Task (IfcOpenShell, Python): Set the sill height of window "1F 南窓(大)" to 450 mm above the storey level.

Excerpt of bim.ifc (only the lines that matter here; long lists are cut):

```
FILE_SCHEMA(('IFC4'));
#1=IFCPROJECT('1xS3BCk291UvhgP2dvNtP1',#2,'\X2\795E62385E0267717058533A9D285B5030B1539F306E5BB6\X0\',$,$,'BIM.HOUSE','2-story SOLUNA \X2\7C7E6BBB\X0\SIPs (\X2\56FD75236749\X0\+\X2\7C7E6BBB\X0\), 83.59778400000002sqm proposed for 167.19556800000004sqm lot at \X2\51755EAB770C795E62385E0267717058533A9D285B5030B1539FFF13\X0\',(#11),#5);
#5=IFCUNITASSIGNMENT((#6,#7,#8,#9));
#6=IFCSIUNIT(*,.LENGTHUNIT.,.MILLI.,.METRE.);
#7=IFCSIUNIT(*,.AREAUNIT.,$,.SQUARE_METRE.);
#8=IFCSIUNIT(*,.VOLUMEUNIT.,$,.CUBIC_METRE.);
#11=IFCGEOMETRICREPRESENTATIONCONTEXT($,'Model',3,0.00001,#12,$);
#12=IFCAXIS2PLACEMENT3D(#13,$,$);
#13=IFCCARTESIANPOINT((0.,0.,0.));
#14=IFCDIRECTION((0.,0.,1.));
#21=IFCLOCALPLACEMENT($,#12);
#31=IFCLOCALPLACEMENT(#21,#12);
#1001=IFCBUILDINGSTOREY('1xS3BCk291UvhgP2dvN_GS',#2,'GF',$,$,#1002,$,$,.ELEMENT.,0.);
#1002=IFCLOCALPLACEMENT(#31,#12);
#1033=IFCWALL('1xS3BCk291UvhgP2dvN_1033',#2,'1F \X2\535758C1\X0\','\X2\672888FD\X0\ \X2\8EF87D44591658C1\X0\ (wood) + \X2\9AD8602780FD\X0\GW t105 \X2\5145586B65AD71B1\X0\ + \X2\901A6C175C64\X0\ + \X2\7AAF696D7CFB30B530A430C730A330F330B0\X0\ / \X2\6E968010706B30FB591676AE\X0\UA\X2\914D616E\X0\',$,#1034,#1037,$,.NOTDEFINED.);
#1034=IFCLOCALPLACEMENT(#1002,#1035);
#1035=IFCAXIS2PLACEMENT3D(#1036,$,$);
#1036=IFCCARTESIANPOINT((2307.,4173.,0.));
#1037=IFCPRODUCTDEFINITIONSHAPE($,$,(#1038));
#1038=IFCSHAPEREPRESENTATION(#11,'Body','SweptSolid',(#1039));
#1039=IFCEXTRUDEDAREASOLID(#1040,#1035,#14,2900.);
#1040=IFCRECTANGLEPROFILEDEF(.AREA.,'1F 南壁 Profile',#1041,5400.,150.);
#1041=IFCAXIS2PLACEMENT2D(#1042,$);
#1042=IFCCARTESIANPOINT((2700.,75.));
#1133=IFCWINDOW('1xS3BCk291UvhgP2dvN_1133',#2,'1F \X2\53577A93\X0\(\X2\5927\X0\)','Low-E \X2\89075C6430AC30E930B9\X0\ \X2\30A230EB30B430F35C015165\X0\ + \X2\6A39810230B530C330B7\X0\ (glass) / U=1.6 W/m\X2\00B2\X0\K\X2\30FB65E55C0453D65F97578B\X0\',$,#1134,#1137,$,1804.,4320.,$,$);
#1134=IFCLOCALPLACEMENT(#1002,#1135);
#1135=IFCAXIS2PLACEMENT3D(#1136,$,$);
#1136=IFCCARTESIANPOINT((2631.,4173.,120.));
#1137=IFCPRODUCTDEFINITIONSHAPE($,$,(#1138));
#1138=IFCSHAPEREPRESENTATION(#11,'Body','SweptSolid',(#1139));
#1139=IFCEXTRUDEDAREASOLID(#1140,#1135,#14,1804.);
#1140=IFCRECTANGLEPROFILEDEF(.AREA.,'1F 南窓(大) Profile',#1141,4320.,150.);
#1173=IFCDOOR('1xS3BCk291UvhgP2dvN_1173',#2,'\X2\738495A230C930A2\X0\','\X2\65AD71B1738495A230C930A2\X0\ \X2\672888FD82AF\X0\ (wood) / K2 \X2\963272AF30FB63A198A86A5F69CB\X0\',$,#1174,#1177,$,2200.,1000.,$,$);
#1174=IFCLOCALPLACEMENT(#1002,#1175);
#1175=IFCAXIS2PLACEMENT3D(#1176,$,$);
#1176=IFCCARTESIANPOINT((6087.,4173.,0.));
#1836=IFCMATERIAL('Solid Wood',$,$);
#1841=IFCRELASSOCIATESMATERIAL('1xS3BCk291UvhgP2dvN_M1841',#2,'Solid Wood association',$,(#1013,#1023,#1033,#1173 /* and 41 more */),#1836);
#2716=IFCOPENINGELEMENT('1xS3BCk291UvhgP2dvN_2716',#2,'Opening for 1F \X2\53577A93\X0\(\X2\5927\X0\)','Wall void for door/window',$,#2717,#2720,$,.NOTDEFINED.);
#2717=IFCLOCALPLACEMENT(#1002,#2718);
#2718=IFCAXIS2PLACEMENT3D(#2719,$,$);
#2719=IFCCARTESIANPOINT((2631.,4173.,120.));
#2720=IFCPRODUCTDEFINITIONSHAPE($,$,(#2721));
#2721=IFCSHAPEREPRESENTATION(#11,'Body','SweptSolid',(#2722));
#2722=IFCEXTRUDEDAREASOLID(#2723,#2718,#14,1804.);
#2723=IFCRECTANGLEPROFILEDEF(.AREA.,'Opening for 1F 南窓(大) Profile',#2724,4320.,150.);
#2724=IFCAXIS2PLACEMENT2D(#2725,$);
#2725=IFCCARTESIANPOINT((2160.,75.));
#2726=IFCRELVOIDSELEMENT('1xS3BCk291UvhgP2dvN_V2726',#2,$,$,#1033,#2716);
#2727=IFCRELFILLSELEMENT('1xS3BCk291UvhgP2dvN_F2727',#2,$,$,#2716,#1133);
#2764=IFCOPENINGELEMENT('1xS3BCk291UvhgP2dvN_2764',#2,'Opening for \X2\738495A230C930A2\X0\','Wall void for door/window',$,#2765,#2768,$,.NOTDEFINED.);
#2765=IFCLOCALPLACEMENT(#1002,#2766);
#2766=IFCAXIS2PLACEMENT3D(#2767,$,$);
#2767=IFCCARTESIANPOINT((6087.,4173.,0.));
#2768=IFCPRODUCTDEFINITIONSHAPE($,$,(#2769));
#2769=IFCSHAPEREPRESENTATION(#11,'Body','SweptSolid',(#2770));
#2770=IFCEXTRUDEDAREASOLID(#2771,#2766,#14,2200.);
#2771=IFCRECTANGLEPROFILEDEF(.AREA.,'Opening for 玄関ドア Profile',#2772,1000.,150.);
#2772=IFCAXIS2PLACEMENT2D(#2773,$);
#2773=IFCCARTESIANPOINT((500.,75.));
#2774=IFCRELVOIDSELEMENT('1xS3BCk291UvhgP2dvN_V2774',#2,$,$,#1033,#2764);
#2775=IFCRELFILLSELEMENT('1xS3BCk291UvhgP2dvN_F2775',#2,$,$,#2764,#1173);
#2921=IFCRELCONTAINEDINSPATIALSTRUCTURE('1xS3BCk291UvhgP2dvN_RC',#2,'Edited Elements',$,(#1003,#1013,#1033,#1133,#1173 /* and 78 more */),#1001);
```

```python
import numpy as np
import ifcopenshell
import ifcopenshell.api.geometry
import ifcopenshell.geom
import ifcopenshell.util.element
import ifcopenshell.util.placement
import ifcopenshell.util.shape
import ifcopenshell.util.unit

model = ifcopenshell.open("bim.ifc")
unit_scale = ifcopenshell.util.unit.calculate_unit_scale(model)

window = model.by_id(1133)
opening = window.FillsVoids[0].RelatingOpeningElement
storey = ifcopenshell.util.element.get_container(window, ifc_class="IfcBuildingStorey")
level = ifcopenshell.util.placement.get_local_placement(storey.ObjectPlacement)[2, 3]

# The opening's origin need not be at the sill, so measure its lowest point.
shape = ifcopenshell.geom.create_shape(ifcopenshell.geom.settings(), opening)
bottom = ifcopenshell.util.shape.get_shape_bottom_elevation(shape, shape.geometry) / unit_scale
dz = level + 0.45 / unit_scale - bottom

shift = np.array([0.0, 0.0, dz])
# The window is not placed relative to its opening, so move both.
for product in (opening, window):
    matrix = ifcopenshell.util.placement.get_local_placement(product.ObjectPlacement)
    matrix[:3, 3] += shift
    ifcopenshell.api.geometry.edit_object_placement(model, product=product, matrix=matrix, is_si=False)

print(f"moved by {dz * unit_scale:+.3f} m")

model.write("bim_rev.ifc")
```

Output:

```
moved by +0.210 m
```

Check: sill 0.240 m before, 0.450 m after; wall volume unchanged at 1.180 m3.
